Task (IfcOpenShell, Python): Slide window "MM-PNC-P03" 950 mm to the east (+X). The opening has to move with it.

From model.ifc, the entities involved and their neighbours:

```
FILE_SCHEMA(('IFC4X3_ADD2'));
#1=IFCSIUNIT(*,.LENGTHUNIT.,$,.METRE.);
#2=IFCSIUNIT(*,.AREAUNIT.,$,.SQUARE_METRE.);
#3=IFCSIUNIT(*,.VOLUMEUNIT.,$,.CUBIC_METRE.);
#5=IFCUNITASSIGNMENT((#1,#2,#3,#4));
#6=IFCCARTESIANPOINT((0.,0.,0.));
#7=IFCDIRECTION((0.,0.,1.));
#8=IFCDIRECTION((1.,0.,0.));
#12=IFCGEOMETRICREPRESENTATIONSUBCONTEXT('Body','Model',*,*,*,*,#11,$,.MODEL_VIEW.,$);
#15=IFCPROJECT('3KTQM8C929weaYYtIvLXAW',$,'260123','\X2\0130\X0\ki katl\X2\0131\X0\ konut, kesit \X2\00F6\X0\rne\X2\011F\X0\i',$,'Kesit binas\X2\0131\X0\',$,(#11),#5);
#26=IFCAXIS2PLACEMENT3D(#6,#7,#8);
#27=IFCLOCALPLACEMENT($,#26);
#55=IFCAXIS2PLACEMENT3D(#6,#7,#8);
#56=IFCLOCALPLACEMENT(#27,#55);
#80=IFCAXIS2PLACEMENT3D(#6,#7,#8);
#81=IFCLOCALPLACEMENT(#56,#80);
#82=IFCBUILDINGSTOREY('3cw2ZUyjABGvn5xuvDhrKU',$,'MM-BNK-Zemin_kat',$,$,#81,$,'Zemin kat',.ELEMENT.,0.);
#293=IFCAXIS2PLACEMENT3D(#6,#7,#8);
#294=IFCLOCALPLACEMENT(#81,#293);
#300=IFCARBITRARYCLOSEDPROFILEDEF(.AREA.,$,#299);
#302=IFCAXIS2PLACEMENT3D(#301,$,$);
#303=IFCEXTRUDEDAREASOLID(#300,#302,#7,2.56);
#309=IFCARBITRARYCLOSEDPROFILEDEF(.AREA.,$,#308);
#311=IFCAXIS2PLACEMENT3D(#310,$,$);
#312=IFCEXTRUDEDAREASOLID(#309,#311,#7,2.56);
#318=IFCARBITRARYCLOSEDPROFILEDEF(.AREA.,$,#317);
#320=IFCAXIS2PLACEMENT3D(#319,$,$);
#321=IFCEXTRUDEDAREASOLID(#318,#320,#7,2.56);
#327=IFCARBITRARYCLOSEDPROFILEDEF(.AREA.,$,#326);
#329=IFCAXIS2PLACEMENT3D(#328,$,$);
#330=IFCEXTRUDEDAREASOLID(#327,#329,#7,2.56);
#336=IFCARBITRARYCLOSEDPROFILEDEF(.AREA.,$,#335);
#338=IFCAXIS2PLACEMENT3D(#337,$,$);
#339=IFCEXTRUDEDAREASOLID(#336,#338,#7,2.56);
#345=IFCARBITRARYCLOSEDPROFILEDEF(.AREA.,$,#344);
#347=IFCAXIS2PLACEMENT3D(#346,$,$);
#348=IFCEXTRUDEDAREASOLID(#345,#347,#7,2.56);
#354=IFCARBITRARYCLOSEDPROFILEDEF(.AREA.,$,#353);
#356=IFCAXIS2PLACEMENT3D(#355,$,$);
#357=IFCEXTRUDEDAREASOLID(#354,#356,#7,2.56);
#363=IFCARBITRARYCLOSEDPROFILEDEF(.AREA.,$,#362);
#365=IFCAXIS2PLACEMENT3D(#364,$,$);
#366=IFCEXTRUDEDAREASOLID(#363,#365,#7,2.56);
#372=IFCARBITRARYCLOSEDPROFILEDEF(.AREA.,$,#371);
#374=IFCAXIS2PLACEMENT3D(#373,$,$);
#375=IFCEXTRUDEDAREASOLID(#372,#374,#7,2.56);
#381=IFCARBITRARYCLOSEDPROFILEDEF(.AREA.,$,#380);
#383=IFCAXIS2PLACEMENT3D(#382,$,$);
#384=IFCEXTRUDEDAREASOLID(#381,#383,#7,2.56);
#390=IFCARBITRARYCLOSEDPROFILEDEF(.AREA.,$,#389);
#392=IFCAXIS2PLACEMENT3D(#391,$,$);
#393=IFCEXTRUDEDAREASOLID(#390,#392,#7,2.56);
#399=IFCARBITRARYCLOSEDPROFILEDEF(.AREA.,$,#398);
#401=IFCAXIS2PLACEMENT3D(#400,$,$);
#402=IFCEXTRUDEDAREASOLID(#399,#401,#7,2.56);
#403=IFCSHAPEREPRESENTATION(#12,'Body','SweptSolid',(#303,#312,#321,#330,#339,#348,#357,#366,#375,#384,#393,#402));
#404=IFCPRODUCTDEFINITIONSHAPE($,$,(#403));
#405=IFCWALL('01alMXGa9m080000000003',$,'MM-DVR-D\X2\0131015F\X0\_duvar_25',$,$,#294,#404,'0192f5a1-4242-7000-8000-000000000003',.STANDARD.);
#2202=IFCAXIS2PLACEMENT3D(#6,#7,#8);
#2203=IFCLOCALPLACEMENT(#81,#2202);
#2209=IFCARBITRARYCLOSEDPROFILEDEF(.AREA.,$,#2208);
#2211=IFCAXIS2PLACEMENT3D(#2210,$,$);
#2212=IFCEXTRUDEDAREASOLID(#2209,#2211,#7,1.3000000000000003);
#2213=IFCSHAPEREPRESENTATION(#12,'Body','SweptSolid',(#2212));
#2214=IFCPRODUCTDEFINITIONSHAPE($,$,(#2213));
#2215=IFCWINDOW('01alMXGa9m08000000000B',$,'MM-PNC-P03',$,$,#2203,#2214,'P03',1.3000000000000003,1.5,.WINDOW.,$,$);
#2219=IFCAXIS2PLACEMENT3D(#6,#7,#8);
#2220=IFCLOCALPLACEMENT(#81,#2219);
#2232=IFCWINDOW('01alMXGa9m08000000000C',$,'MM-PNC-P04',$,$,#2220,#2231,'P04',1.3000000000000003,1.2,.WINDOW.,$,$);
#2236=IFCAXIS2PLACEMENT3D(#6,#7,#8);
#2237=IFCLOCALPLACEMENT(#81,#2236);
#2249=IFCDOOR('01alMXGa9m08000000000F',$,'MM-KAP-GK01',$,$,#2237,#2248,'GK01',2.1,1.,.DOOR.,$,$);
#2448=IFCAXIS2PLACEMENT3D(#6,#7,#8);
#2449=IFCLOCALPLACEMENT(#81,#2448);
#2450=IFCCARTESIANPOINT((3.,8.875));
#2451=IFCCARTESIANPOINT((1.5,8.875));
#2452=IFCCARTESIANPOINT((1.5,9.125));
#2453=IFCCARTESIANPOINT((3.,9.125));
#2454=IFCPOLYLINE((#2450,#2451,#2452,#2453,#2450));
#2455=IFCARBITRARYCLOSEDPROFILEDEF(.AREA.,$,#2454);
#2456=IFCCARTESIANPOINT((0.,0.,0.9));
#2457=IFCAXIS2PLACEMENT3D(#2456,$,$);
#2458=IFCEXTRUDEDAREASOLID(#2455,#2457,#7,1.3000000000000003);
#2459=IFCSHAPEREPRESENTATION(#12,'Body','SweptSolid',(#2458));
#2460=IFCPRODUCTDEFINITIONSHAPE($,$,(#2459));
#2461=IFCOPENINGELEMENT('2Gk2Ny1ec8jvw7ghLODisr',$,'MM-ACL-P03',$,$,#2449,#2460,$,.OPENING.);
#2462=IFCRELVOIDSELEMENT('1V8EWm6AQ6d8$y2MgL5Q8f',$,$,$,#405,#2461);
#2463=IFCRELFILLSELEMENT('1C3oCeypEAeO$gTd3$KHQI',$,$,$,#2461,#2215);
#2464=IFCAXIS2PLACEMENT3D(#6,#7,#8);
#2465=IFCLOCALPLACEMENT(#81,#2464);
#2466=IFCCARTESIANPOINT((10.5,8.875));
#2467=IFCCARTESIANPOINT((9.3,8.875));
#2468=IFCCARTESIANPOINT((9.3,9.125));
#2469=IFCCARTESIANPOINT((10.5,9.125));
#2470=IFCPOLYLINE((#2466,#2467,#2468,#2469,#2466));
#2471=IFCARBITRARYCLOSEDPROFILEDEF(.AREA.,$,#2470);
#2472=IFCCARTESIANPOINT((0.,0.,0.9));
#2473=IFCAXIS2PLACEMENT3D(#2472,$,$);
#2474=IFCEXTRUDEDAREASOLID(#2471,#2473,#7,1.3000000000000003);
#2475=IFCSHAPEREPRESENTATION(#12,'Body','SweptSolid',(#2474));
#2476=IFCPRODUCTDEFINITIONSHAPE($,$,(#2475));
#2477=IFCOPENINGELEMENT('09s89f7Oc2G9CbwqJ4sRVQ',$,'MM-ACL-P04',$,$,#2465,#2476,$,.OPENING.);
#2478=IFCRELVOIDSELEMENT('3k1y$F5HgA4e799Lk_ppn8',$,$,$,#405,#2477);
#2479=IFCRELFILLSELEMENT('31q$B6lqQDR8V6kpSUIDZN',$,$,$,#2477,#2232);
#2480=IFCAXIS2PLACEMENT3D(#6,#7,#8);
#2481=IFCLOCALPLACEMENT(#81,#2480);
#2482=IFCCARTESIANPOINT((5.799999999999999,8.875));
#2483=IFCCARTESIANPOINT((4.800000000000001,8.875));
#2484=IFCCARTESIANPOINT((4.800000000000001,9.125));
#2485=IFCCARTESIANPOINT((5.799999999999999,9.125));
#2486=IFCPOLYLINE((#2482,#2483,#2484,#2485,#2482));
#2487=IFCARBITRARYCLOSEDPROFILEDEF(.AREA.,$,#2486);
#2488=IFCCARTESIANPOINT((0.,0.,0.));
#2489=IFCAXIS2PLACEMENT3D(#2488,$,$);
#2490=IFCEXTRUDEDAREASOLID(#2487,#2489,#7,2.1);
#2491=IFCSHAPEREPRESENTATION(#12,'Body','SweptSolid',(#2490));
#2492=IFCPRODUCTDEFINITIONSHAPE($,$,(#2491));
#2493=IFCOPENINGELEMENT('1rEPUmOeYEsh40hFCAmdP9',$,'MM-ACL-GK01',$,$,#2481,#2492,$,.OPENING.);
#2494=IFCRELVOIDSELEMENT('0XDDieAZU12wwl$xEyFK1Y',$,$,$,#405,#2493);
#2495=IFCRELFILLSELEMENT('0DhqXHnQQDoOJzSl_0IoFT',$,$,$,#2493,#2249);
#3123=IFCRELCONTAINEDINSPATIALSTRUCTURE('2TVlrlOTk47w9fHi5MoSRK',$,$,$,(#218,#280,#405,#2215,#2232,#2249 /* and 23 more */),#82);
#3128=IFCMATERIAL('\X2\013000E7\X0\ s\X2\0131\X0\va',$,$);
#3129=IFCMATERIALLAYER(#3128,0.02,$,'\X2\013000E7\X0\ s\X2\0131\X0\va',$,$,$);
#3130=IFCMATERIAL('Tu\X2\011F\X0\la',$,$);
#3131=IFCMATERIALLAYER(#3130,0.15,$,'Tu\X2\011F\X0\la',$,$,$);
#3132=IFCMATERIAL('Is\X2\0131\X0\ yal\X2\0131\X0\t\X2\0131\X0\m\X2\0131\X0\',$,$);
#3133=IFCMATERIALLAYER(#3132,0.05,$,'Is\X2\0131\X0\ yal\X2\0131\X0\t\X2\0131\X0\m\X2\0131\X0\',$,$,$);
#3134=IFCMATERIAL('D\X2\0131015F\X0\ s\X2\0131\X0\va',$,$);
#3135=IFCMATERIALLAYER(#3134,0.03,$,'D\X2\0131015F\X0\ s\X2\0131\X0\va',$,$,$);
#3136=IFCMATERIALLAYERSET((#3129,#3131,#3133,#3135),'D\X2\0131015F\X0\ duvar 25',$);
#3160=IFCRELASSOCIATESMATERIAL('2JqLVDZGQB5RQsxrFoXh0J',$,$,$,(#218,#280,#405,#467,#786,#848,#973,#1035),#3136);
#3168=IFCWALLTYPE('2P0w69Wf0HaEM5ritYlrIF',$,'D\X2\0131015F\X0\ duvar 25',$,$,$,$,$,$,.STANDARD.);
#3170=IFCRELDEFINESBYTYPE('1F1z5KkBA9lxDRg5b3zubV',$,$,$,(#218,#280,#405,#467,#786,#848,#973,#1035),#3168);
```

```python
import ifcopenshell
import ifcopenshell.api.geometry
import ifcopenshell.util.placement

model = ifcopenshell.open("model.ifc")

window = model.by_id(2215)
opening = window.FillsVoids[0].RelatingOpeningElement
wall = opening.VoidsElements[0].RelatingBuildingElement

wall_matrix = ifcopenshell.util.placement.get_local_placement(wall.ObjectPlacement)
shift = wall_matrix[:3, 0] * 0.95
before = ifcopenshell.util.placement.get_local_placement(window.ObjectPlacement)[:3, 3].copy()

# The window is not placed relative to its opening, so move both.
for product in (opening, window):
    matrix = ifcopenshell.util.placement.get_local_placement(product.ObjectPlacement)
    matrix[:3, 3] += shift
    ifcopenshell.api.geometry.edit_object_placement(model, product=product, matrix=matrix, is_si=False)

after = ifcopenshell.util.placement.get_local_placement(window.ObjectPlacement)[:3, 3]
print("window moved by", (after - before).round(3) + 0.0)

model.write("model_updated.ifc")
```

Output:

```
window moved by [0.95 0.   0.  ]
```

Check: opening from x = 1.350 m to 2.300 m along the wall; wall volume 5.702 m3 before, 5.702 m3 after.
